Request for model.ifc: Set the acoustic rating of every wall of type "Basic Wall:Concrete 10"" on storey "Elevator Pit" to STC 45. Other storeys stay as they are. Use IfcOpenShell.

First a look at what the model holds.

```python
import ifcopenshell
import ifcopenshell.util.element

model = ifcopenshell.open("model.ifc")
print(model.schema)
storey = next(s for s in model.by_type("IfcBuildingStorey") if s.Name == "Elevator Pit")
walls = [e for e in ifcopenshell.util.element.get_decomposition(storey) if e.is_a("IfcWall")]
seen = {}
for e in walls:
    element_type = ifcopenshell.util.element.get_type(e)
    key = (element_type.Name if element_type != e and element_type else None, ifcopenshell.util.element.get_pset(e, "Pset_WallCommon", "AcousticRating"))
    seen[key] = seen.get(key, 0) + 1
for (name, value), count in sorted(seen.items(), key=str):
    print(count, "x", name, "|", value)
```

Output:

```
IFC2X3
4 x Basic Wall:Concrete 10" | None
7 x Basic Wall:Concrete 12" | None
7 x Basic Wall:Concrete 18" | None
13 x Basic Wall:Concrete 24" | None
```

```python
import ifcopenshell
import ifcopenshell.api.pset
import ifcopenshell.util.element

model = ifcopenshell.open("model.ifc")

storey = next(s for s in model.by_type("IfcBuildingStorey") if s.Name == "Elevator Pit")
walls = [e for e in ifcopenshell.util.element.get_decomposition(storey) if e.is_a("IfcWall")]

count = 0
for e in walls:
    element_type = ifcopenshell.util.element.get_type(e)
    if element_type in (None, e) or element_type.Name != 'Basic Wall:Concrete 10"':
        continue
    # add_pset returns the element's existing set when there is one.
    pset = ifcopenshell.api.pset.add_pset(model, product=e, name="Pset_WallCommon")
    ifcopenshell.api.pset.edit_pset(model, pset=pset, properties={"AcousticRating": "STC 45"})
    count += 1

print(count, "walls updated")

model.write("model_updated.ifc")
```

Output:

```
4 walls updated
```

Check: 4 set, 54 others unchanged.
